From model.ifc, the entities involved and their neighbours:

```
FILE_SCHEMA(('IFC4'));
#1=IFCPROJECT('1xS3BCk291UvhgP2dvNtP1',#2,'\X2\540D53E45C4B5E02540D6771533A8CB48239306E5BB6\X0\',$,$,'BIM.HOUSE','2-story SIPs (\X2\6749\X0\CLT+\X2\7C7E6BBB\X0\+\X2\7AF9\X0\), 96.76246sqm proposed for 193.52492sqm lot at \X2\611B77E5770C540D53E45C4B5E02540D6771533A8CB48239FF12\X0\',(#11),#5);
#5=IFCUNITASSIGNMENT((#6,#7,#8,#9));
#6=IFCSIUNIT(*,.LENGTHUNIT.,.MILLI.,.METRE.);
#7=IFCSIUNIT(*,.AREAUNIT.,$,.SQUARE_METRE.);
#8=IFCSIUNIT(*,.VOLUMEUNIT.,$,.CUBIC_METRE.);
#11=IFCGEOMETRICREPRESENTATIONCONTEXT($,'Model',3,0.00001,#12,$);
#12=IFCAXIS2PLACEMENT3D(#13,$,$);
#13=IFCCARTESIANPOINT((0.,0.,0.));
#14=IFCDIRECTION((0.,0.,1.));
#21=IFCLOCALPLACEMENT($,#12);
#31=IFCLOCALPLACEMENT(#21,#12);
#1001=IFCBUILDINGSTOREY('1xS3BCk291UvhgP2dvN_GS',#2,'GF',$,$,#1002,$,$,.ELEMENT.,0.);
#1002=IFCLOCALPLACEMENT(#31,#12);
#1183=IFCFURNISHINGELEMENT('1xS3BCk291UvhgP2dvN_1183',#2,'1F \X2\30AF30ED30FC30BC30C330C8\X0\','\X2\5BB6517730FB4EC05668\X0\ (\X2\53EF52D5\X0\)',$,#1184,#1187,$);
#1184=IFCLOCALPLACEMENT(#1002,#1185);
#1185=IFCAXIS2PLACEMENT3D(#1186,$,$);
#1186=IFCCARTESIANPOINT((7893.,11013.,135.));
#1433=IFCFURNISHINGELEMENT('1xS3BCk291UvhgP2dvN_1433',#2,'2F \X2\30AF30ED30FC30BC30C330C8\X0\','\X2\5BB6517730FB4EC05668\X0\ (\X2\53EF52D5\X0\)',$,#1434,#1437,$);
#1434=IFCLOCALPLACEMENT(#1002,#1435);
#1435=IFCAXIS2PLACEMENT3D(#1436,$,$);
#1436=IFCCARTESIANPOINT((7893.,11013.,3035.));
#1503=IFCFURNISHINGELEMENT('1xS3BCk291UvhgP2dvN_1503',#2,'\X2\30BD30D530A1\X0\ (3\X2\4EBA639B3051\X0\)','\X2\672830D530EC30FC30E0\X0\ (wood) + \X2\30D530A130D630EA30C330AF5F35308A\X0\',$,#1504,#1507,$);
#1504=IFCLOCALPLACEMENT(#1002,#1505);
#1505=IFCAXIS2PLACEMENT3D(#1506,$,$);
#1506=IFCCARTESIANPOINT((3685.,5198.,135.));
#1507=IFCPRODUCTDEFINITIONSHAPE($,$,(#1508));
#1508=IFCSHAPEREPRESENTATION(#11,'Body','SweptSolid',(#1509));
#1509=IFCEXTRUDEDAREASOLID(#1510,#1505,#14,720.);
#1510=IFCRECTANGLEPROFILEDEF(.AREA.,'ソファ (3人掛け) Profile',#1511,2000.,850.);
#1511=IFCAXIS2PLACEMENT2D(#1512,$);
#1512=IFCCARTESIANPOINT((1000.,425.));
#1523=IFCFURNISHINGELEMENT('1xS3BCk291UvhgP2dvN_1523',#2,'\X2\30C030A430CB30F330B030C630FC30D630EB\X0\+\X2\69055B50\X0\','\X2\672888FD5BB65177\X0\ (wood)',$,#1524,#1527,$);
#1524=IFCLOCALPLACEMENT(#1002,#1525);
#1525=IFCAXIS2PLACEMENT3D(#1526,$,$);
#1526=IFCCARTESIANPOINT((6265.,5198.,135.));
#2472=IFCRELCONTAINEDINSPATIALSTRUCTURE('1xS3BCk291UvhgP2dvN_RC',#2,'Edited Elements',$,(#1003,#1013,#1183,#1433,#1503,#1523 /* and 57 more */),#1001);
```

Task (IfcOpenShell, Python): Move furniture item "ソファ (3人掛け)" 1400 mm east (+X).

```python
import ifcopenshell
import ifcopenshell.api.geometry
import ifcopenshell.util.placement
import ifcopenshell.util.unit

model = ifcopenshell.open("model.ifc")
unit_scale = ifcopenshell.util.unit.calculate_unit_scale(model)

item = model.by_guid("1xS3BCk291UvhgP2dvN_1503")
matrix = ifcopenshell.util.placement.get_local_placement(item.ObjectPlacement)
matrix[0, 3] += 1.4 / unit_scale
ifcopenshell.api.geometry.edit_object_placement(model, product=item, matrix=matrix, is_si=False)

print(ifcopenshell.util.placement.get_local_placement(item.ObjectPlacement).round(3) + 0.0)

model.write("model_v2.ifc")
```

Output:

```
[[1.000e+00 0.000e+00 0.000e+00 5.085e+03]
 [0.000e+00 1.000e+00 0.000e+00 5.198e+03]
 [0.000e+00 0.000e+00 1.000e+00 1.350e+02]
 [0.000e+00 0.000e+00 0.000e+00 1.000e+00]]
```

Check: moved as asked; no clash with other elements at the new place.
